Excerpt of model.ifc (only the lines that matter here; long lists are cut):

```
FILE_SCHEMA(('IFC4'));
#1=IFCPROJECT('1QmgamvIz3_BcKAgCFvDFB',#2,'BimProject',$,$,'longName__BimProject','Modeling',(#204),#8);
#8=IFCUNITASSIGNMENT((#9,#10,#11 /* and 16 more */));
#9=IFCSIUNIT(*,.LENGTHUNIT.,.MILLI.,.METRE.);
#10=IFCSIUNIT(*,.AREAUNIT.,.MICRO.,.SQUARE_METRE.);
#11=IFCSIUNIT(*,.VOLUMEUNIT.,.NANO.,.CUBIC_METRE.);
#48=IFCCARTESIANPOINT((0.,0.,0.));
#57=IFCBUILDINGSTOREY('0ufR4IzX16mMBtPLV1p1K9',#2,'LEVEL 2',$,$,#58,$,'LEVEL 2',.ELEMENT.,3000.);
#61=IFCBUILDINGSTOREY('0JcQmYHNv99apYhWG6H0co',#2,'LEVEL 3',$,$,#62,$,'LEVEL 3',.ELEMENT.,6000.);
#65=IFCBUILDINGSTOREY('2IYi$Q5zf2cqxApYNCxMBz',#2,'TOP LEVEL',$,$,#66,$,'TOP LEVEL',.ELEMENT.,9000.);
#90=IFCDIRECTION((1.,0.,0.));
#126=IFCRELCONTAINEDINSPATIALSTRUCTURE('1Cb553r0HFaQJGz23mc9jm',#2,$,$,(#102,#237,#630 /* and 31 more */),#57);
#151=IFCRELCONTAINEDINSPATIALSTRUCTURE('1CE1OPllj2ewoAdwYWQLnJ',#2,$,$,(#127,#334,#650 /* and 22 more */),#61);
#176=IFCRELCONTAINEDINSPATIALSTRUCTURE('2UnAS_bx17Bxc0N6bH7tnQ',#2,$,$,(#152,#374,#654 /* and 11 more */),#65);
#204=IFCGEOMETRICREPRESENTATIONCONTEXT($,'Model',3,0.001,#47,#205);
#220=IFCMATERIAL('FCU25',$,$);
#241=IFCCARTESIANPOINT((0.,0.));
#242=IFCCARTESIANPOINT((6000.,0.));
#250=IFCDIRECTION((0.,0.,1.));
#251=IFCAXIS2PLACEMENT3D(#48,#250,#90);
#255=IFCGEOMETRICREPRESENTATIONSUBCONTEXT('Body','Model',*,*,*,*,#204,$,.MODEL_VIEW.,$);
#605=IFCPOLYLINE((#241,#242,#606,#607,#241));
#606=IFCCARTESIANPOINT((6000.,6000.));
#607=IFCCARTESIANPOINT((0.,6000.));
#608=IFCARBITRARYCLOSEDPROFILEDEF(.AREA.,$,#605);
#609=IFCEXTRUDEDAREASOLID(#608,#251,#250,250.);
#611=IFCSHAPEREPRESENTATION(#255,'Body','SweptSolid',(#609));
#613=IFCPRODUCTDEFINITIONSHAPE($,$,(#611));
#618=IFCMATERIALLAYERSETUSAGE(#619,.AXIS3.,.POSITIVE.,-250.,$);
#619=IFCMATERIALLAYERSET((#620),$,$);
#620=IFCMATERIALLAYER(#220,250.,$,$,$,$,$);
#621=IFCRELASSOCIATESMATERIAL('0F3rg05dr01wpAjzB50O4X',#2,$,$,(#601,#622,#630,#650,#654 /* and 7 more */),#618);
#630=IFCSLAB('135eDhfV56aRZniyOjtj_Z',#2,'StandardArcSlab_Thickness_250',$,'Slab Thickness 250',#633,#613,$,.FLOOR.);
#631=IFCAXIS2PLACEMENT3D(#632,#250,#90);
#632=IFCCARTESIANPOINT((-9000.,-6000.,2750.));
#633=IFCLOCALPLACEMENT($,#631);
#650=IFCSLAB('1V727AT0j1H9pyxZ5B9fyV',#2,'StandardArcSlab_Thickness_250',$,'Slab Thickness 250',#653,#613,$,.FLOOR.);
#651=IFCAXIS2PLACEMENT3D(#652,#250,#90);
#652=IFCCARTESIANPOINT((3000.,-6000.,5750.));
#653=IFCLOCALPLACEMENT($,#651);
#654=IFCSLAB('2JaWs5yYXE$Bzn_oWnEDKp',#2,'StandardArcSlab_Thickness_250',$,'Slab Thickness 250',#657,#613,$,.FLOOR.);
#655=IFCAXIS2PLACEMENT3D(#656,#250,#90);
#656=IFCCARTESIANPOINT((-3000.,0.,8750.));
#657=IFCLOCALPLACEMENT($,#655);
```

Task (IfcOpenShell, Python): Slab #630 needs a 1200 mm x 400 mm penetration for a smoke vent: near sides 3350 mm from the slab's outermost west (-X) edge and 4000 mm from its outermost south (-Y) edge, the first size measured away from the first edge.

```python
import numpy as np
import ifcopenshell
import ifcopenshell.api.feature
import ifcopenshell.api.geometry
import ifcopenshell.api.root
import ifcopenshell.geom
import ifcopenshell.util.placement
import ifcopenshell.util.representation
import ifcopenshell.util.shape
import ifcopenshell.util.unit

model = ifcopenshell.open("model.ifc")
unit_scale = ifcopenshell.util.unit.calculate_unit_scale(model)
settings = ifcopenshell.geom.settings()


def volume(element):
    """Net volume in cubic metres, openings subtracted."""
    shape = ifcopenshell.geom.create_shape(settings, element)
    return ifcopenshell.util.shape.get_volume(shape.geometry)


slab = model.by_guid("135eDhfV56aRZniyOjtj_Z")
before = volume(slab)

# Extent in the slab's own axes, in metres. The edges named are its -X and -Y sides.
slab_shape = ifcopenshell.geom.create_shape(settings, slab)
vertices = ifcopenshell.util.shape.get_vertices(slab_shape.geometry)
x_min, y_min, bottom = vertices.min(axis=0)
top = vertices[:, 2].max()

opening = ifcopenshell.api.root.create_entity(model, ifc_class="IfcOpeningElement", name="Smoke vent opening", predefined_type="OPENING")
context = ifcopenshell.util.representation.get_context(model, "Model", "Body", "MODEL_VIEW")
width, depth = 1.2, 0.4
outline = [(0.0, 0.0), (width, 0.0), (width, depth), (0.0, depth), (0.0, 0.0)]
# Overshoot both faces by 50 mm so the cut is clean.
shape = ifcopenshell.api.geometry.add_slab_representation(
    model, context=context, depth=top - bottom + 0.1, polyline=outline
)
ifcopenshell.api.geometry.assign_representation(model, product=opening, representation=shape)

matrix = ifcopenshell.util.placement.get_local_placement(slab.ObjectPlacement)
matrix[:, 3] = matrix @ np.append(np.array([x_min + 3.35, y_min + 4, bottom - 0.05]) / unit_scale, 1.0)
ifcopenshell.api.geometry.edit_object_placement(model, product=opening, matrix=matrix, is_si=False)
ifcopenshell.api.feature.add_feature(model, feature=opening, element=slab)

after = volume(slab)

print(f"slab volume {before:.3f} -> {after:.3f} m3")

model.write("model-out.ifc")
```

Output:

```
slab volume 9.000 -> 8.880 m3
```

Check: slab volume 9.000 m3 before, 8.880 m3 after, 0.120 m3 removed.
